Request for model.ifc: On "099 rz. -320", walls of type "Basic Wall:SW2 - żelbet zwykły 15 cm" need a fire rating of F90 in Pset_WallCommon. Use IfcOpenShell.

First a look at what the model holds.

```python
import ifcopenshell
import ifcopenshell.util.element

model = ifcopenshell.open("model.ifc")
print(model.schema)
storey = next(s for s in model.by_type("IfcBuildingStorey") if s.Name == "099 rz. -320")
walls = [e for e in ifcopenshell.util.element.get_decomposition(storey) if e.is_a("IfcWall")]
seen = {}
for e in walls:
    element_type = ifcopenshell.util.element.get_type(e)
    key = (element_type.Name if element_type != e and element_type else None, ifcopenshell.util.element.get_pset(e, "Pset_WallCommon", "FireRating"))
    seen[key] = seen.get(key, 0) + 1
for (name, value), count in sorted(seen.items(), key=str):
    print(count, "x", name, "|", value)
```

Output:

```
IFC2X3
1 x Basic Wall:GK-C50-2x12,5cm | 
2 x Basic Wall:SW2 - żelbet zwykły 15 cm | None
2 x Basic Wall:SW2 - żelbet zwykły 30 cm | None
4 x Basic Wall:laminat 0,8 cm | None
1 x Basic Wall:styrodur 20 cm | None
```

```python
import ifcopenshell
import ifcopenshell.api.pset
import ifcopenshell.util.element

model = ifcopenshell.open("model.ifc")

storey = next(s for s in model.by_type("IfcBuildingStorey") if s.Name == "099 rz. -320")
walls = [e for e in ifcopenshell.util.element.get_decomposition(storey) if e.is_a("IfcWall")]

count = 0
for e in walls:
    element_type = ifcopenshell.util.element.get_type(e)
    if element_type in (None, e) or element_type.Name != "Basic Wall:SW2 - żelbet zwykły 15 cm":
        continue
    # add_pset returns the element's existing set when there is one.
    pset = ifcopenshell.api.pset.add_pset(model, product=e, name="Pset_WallCommon")
    ifcopenshell.api.pset.edit_pset(model, pset=pset, properties={"FireRating": "F90"})
    count += 1

print(count, "walls updated")

model.write("model_v2.ifc")
```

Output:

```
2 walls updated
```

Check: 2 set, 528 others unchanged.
